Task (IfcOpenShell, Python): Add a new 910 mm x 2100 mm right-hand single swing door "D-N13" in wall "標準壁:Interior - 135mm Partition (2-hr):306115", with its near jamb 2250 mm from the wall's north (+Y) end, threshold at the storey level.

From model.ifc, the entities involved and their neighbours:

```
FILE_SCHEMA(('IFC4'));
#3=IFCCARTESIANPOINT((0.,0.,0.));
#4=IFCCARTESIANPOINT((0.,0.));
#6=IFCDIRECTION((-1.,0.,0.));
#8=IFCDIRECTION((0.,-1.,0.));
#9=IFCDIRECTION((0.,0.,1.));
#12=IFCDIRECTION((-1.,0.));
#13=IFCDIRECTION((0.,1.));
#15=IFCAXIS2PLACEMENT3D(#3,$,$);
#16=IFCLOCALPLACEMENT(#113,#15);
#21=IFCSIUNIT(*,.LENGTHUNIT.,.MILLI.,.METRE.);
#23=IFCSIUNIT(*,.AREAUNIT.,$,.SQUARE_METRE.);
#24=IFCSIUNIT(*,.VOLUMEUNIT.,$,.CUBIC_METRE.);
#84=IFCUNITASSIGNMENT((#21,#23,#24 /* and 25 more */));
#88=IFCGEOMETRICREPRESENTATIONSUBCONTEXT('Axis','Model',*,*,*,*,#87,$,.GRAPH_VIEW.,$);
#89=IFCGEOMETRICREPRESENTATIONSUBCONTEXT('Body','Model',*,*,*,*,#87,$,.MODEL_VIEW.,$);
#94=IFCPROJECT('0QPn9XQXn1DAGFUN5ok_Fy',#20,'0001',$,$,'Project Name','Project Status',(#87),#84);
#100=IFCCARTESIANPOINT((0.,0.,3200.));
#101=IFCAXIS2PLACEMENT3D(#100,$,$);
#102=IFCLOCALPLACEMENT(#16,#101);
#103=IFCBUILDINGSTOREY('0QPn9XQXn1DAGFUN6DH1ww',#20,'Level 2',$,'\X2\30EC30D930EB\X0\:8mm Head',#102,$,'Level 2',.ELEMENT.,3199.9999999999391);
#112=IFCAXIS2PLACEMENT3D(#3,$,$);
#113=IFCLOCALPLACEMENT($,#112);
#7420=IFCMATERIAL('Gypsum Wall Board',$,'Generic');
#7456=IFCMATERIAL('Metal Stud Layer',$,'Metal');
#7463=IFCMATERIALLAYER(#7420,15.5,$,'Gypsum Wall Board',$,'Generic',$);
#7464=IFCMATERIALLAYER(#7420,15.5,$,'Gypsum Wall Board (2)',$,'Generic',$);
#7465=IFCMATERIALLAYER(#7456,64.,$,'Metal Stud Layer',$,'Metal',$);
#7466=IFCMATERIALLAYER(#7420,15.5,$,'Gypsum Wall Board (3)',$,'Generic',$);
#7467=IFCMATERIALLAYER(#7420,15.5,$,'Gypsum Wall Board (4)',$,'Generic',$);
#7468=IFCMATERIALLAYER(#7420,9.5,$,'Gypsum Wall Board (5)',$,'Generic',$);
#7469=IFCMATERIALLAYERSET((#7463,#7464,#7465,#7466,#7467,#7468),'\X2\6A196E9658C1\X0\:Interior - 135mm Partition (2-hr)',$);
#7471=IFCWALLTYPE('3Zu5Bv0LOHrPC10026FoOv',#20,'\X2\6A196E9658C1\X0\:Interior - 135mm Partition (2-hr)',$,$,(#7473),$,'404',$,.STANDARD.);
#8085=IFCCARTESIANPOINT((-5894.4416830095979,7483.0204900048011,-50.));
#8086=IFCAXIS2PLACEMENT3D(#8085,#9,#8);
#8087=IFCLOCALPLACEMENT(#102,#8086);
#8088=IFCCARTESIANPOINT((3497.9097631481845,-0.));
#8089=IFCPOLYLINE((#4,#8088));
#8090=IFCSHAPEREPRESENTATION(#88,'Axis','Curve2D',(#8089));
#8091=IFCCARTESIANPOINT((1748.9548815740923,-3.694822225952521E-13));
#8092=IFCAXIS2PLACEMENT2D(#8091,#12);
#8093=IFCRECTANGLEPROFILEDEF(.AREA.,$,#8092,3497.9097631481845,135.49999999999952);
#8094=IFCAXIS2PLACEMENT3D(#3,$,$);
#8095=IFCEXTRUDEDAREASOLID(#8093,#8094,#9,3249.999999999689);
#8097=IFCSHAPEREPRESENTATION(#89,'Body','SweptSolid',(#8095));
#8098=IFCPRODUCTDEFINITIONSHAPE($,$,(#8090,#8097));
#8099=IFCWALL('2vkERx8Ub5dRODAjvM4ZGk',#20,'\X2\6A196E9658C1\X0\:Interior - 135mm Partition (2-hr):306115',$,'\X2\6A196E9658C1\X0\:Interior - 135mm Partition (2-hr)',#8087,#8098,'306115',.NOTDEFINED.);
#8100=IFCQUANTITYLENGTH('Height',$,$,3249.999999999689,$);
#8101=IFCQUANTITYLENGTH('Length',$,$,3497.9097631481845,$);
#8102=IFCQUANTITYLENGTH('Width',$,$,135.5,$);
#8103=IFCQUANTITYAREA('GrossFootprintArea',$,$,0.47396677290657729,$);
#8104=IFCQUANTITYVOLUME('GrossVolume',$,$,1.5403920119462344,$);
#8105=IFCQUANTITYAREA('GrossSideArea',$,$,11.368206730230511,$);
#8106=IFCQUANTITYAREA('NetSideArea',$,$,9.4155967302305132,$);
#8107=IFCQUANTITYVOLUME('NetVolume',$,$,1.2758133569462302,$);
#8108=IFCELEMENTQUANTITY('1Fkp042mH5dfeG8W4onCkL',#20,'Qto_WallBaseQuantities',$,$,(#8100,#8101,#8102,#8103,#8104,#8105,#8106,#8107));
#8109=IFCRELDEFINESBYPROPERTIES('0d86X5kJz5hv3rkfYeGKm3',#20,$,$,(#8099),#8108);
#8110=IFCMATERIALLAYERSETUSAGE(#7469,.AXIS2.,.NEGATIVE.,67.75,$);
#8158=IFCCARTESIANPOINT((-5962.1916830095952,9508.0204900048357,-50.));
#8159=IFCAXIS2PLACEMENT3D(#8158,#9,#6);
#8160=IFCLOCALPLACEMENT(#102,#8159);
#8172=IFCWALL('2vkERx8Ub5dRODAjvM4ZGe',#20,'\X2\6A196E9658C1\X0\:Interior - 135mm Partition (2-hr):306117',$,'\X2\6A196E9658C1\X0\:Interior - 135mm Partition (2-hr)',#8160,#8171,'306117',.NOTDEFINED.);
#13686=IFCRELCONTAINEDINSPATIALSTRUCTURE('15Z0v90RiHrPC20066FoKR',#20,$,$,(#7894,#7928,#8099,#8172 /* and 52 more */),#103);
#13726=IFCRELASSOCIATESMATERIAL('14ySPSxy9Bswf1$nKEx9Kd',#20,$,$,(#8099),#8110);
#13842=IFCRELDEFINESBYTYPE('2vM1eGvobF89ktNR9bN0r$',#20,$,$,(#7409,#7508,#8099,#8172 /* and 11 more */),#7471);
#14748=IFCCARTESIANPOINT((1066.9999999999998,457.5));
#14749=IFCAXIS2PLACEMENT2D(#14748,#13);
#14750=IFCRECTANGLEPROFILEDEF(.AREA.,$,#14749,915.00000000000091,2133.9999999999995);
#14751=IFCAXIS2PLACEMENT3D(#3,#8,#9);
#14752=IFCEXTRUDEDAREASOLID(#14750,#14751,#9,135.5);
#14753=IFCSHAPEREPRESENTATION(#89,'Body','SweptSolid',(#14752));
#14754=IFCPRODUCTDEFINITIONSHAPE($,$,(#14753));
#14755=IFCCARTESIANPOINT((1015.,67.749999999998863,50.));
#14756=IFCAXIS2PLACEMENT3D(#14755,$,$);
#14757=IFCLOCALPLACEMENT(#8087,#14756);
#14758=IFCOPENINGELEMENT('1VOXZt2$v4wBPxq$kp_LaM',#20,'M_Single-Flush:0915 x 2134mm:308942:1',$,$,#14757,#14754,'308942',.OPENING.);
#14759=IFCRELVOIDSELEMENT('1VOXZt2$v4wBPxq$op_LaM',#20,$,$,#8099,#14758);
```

```python
import numpy as np
import ifcopenshell
import ifcopenshell.api.feature
import ifcopenshell.api.geometry
import ifcopenshell.api.pset
import ifcopenshell.api.root
import ifcopenshell.api.spatial
import ifcopenshell.geom
import ifcopenshell.util.element
import ifcopenshell.util.placement
import ifcopenshell.util.representation
import ifcopenshell.util.shape
import ifcopenshell.util.unit

model = ifcopenshell.open("model.ifc")
unit_scale = ifcopenshell.util.unit.calculate_unit_scale(model)
area_scale = ifcopenshell.util.unit.calculate_unit_scale(model, "AREAUNIT")
volume_scale = ifcopenshell.util.unit.calculate_unit_scale(model, "VOLUMEUNIT")
settings = ifcopenshell.geom.settings()


def volume(element):
    """Net volume in cubic metres, openings subtracted."""
    shape = ifcopenshell.geom.create_shape(settings, element)
    return ifcopenshell.util.shape.get_volume(shape.geometry)


wall = model.by_id(8099)
storey = ifcopenshell.util.element.get_container(wall, ifc_class="IfcBuildingStorey")
context = ifcopenshell.util.representation.get_context(model, "Model", "Body", "MODEL_VIEW")
before = volume(wall)

width, height, from_end, sill = 0.91, 2.1, 2.25, 0.0  # metres

# The wall runs along its own X axis, and the end named is its -X end.
wall_shape = ifcopenshell.geom.create_shape(settings, wall)
x, y, z = ifcopenshell.util.shape.get_vertices(wall_shape.geometry).T
start = x.min() + from_end
face, thickness = float(y.min()), float(y.max() - y.min())
wall_matrix = ifcopenshell.util.placement.get_local_placement(wall.ObjectPlacement)
level = ifcopenshell.util.placement.get_local_placement(storey.ObjectPlacement)[2, 3]


def in_wall(x, y):
    """Placement at x, y metres in the wall's axes, at sill height."""
    matrix = wall_matrix.copy()
    matrix[:, 3] = wall_matrix @ np.array([x / unit_scale, y / unit_scale, 0.0, 1.0])
    matrix[2, 3] = level + sill / unit_scale
    return matrix


# Opening: a box that overshoots both wall faces by 50 mm.
opening = ifcopenshell.api.root.create_entity(model, ifc_class="IfcOpeningElement", predefined_type="OPENING")
box = ifcopenshell.api.geometry.add_wall_representation(
    model, context=context, length=width, height=height, thickness=thickness + 0.1
)
ifcopenshell.api.geometry.assign_representation(model, product=opening, representation=box)
ifcopenshell.api.geometry.edit_object_placement(model, product=opening, matrix=in_wall(start, face - 0.05), is_si=False)
ifcopenshell.api.feature.add_feature(model, feature=opening, element=wall)

door = ifcopenshell.api.root.create_entity(model, ifc_class="IfcDoor", name="D-N13", predefined_type="DOOR")
door.OverallWidth, door.OverallHeight = width / unit_scale, height / unit_scale
door.OperationType = "SINGLE_SWING_RIGHT"
body = ifcopenshell.api.geometry.add_door_representation(
    model,
    context=context,
    overall_width=door.OverallWidth,
    overall_height=door.OverallHeight,
    operation_type="SINGLE_SWING_RIGHT",
    lining_properties={"LiningDepth": thickness / unit_scale, "ThresholdDepth": thickness / unit_scale},
)
ifcopenshell.api.geometry.assign_representation(model, product=door, representation=body)
ifcopenshell.api.spatial.assign_container(model, products=[door], relating_structure=storey)
ifcopenshell.api.feature.add_filling(model, opening=opening, element=door)

# The lining spans the wall, so the door starts at the wall face.
ifcopenshell.api.geometry.edit_object_placement(model, product=door, matrix=in_wall(start, face), is_si=False)

after = volume(wall)

# Update the wall's stored quantities.
qto = model.by_id(ifcopenshell.util.element.get_pset(wall, "Qto_WallBaseQuantities", should_inherit=False)["id"])
ifcopenshell.api.pset.edit_qto(model, qto=qto, properties={
    "NetSideArea": after / thickness / area_scale,
    "NetVolume": after / volume_scale,
})

print(f"wall volume {before:.3f} -> {after:.3f} m3")

model.write("model_v2.ifc")
```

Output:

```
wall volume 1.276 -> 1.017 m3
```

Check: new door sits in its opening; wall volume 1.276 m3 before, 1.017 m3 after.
